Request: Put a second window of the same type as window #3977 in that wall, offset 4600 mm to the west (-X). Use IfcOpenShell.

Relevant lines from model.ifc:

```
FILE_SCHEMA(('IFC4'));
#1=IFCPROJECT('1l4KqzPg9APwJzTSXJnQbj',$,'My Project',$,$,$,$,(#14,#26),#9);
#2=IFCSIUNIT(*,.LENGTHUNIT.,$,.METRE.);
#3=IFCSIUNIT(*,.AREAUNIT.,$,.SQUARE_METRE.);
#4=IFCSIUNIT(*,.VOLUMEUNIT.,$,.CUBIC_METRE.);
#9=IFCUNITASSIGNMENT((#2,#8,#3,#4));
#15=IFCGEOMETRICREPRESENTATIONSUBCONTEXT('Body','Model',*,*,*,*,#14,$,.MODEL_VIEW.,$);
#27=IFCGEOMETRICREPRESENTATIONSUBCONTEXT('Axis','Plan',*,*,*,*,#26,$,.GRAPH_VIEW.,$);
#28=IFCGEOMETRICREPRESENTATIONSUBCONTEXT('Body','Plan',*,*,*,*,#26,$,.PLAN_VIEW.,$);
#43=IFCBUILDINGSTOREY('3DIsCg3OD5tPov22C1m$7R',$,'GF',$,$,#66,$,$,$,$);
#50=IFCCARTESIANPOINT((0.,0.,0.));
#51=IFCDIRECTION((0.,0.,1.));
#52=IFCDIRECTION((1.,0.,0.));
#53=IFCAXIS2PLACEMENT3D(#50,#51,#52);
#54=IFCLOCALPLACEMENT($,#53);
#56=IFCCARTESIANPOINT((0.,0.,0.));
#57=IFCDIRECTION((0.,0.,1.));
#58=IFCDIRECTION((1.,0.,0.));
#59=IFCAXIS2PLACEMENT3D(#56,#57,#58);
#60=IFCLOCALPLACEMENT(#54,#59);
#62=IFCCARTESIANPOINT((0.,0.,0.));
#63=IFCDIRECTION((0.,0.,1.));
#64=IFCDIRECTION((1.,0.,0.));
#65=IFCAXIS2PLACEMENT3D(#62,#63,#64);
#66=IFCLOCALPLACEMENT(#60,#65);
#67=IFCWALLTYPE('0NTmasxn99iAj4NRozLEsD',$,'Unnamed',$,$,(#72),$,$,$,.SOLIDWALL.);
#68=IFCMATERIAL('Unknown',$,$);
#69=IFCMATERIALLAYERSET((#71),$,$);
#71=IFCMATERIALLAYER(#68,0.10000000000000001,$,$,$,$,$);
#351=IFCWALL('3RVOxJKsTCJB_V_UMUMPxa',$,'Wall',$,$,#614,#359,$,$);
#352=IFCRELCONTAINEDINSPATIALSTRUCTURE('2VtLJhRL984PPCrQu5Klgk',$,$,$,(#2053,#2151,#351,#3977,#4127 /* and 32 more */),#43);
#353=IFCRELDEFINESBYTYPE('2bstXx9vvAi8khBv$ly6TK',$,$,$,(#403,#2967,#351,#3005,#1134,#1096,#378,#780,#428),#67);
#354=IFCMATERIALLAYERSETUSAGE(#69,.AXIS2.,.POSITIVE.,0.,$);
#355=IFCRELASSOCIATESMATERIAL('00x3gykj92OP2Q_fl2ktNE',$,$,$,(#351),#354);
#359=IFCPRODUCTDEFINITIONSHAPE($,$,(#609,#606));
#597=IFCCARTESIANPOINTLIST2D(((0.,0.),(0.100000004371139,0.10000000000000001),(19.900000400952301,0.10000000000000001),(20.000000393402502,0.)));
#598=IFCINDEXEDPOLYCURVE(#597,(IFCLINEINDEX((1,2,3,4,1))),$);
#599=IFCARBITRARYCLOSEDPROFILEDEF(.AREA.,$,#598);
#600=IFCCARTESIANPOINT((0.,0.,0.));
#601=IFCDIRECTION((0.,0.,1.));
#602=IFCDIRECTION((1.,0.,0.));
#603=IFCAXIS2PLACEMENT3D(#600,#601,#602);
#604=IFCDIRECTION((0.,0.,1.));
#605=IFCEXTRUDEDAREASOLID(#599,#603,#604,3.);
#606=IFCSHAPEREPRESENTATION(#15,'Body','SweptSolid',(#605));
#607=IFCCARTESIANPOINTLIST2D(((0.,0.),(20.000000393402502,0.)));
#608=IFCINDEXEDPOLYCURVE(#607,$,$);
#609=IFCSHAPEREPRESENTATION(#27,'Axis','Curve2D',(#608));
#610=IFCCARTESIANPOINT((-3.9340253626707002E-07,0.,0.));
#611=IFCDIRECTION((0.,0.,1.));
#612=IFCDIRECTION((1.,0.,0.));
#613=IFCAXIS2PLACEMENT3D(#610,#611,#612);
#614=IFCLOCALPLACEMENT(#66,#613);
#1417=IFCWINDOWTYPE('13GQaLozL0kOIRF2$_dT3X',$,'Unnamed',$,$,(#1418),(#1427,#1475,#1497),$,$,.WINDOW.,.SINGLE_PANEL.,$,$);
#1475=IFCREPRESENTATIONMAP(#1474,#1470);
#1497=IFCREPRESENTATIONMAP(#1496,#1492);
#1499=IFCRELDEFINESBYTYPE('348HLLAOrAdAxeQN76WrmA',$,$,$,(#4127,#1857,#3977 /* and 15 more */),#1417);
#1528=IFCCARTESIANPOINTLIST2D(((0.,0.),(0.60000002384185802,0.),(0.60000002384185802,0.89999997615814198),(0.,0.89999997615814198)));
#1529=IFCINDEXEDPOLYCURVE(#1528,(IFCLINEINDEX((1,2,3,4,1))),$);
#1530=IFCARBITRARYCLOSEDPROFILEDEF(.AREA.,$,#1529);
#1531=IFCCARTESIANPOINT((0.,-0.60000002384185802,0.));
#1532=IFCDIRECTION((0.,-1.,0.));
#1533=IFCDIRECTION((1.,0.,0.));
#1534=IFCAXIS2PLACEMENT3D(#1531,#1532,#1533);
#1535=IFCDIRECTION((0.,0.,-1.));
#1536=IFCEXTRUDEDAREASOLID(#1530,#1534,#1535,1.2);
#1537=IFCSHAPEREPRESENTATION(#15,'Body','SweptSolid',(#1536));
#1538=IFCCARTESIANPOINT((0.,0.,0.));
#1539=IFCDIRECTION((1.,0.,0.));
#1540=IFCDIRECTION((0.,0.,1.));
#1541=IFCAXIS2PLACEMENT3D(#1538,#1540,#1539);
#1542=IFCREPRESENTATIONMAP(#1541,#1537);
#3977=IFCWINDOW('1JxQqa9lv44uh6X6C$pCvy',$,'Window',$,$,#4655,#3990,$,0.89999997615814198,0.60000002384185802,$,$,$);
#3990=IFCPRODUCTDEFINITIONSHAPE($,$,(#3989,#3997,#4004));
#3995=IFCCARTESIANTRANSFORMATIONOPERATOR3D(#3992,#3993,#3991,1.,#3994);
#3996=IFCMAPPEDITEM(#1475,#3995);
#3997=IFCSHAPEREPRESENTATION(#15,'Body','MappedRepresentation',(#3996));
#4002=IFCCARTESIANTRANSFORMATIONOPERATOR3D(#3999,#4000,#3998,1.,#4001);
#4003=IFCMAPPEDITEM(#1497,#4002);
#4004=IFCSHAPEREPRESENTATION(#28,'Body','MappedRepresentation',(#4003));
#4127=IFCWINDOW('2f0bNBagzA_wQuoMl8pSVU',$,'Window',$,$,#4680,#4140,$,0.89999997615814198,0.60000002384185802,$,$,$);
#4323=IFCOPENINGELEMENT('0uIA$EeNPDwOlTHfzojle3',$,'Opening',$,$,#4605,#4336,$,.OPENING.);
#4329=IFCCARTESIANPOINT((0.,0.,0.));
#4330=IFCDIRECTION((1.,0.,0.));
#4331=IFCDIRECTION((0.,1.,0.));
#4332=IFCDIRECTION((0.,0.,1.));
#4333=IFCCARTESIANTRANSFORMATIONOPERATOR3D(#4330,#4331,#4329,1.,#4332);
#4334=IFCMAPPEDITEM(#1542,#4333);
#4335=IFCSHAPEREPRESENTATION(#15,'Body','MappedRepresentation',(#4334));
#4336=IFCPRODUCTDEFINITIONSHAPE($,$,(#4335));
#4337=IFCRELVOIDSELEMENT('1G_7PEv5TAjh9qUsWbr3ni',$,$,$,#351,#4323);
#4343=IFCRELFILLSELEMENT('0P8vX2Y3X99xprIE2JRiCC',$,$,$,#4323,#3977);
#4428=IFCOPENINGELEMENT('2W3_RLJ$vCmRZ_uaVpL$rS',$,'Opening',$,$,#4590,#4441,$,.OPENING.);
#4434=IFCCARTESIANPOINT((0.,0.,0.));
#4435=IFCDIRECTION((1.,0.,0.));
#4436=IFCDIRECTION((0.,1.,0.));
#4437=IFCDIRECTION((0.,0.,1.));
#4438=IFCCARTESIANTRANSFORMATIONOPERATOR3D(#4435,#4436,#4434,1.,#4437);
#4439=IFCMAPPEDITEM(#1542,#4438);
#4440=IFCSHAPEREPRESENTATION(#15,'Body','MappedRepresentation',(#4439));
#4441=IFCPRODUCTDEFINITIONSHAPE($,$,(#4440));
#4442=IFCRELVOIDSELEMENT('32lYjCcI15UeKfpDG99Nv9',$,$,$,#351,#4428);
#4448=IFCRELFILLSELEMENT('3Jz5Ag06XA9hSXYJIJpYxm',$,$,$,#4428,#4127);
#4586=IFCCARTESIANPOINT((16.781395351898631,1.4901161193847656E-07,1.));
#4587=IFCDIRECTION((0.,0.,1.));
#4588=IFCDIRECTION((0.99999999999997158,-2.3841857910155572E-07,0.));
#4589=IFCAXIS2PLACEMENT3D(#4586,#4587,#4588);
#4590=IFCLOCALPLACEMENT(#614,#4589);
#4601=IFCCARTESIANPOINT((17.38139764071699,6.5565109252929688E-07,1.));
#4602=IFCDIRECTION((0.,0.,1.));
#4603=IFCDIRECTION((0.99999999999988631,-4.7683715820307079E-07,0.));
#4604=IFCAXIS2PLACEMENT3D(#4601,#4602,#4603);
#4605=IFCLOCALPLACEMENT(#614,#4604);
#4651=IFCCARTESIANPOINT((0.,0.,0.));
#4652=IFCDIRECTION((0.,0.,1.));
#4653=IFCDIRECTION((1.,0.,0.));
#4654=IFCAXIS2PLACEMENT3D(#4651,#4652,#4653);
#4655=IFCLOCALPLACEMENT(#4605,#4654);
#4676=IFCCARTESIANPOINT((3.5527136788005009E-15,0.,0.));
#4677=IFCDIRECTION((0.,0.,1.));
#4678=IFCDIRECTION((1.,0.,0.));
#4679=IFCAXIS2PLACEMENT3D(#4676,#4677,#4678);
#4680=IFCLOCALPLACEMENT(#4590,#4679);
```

```python
import ifcopenshell
import ifcopenshell.api.feature
import ifcopenshell.api.geometry
import ifcopenshell.api.root
import ifcopenshell.geom
import ifcopenshell.util.element
import ifcopenshell.util.placement
import ifcopenshell.util.shape
import ifcopenshell.util.unit

model = ifcopenshell.open("model.ifc")
unit_scale = ifcopenshell.util.unit.calculate_unit_scale(model)
settings = ifcopenshell.geom.settings()


def volume(element):
    """Net volume in cubic metres, openings subtracted."""
    shape = ifcopenshell.geom.create_shape(settings, element)
    return ifcopenshell.util.shape.get_volume(shape.geometry)


window = model.by_guid("1JxQqa9lv44uh6X6C$pCvy")
opening = window.FillsVoids[0].RelatingOpeningElement
wall = opening.VoidsElements[0].RelatingBuildingElement
before = volume(wall)
shift = ifcopenshell.util.placement.get_local_placement(wall.ObjectPlacement)[:3, 0] * -4.6 / unit_scale

# copy_class copies the void relationship, type, container and properties, but no geometry.
new_opening = ifcopenshell.api.root.copy_class(model, product=opening)
new_opening.Representation = ifcopenshell.util.element.copy_deep(
    model, opening.Representation, exclude=["IfcGeometricRepresentationContext", "IfcRepresentationMap"]
)
new_window = ifcopenshell.api.root.copy_class(model, product=window)
new_window.Representation = ifcopenshell.util.element.copy_deep(
    model, window.Representation, exclude=["IfcGeometricRepresentationContext", "IfcRepresentationMap"]
)
ifcopenshell.api.feature.add_filling(model, opening=new_opening, element=new_window)

for old, new in ((opening, new_opening), (window, new_window)):
    matrix = ifcopenshell.util.placement.get_local_placement(old.ObjectPlacement)
    matrix[:3, 3] += shift
    ifcopenshell.api.geometry.edit_object_placement(model, product=new, matrix=matrix, is_si=False)

after = volume(wall)

print(f"wall volume {before:.3f} -> {after:.3f} m3")

model.write("model_edited.ifc")
```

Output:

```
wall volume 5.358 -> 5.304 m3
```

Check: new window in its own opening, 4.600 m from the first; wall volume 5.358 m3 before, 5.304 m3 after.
